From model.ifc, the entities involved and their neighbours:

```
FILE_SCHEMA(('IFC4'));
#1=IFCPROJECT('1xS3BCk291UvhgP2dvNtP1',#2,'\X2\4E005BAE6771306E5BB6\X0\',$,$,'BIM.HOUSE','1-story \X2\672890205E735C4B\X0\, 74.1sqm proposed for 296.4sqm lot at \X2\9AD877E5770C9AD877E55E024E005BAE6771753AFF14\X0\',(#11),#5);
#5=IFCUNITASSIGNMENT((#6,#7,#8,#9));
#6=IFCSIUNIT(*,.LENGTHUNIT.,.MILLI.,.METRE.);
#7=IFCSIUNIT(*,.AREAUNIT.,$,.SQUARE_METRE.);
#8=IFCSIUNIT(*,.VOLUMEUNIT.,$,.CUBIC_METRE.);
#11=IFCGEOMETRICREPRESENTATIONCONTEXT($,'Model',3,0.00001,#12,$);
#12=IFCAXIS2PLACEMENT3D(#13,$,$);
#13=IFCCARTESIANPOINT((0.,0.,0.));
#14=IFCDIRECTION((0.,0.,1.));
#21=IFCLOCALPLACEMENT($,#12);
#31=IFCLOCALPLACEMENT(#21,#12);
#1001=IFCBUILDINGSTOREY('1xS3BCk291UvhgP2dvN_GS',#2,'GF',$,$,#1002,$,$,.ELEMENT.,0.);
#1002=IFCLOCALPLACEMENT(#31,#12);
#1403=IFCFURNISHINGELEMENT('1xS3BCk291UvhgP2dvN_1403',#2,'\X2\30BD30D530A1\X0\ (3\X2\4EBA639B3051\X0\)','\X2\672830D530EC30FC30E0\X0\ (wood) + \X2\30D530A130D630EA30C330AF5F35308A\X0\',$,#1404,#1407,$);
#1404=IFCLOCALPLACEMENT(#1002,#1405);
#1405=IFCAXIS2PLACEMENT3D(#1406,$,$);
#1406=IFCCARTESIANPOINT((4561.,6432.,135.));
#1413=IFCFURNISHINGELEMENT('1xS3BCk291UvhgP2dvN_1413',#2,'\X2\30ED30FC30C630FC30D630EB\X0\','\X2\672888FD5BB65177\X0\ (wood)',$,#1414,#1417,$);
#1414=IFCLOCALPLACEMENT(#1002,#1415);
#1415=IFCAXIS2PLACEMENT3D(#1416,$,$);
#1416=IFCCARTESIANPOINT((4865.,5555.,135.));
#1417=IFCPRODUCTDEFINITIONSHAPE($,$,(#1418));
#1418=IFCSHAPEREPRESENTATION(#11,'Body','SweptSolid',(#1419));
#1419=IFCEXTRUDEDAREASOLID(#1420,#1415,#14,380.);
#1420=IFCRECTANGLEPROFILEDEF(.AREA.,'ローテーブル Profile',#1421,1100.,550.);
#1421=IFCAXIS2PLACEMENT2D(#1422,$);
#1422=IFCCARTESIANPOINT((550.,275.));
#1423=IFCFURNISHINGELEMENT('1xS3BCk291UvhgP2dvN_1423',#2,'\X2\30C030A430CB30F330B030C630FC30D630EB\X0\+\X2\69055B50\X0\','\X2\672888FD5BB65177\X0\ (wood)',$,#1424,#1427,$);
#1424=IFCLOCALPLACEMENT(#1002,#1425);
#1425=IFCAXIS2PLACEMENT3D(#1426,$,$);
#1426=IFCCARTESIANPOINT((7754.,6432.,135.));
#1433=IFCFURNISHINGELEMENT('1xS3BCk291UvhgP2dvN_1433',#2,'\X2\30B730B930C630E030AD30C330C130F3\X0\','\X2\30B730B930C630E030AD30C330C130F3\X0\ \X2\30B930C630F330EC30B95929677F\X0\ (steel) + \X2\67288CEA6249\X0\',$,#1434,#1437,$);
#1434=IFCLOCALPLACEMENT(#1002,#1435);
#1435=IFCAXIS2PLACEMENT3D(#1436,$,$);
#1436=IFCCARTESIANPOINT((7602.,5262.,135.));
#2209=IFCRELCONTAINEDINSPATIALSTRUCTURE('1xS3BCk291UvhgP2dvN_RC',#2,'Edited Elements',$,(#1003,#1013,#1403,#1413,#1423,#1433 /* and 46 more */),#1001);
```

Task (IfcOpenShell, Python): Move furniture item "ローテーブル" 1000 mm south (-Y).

```python
import ifcopenshell
import ifcopenshell.api.geometry
import ifcopenshell.util.placement

model = ifcopenshell.open("model.ifc")

item = model.by_guid("1xS3BCk291UvhgP2dvN_1413")
matrix = ifcopenshell.util.placement.get_local_placement(item.ObjectPlacement)
matrix[1, 3] -= 1000.0
ifcopenshell.api.geometry.edit_object_placement(model, product=item, matrix=matrix, is_si=False)

print(ifcopenshell.util.placement.get_local_placement(item.ObjectPlacement).round(3) + 0.0)

model.write("model_rev.ifc")
```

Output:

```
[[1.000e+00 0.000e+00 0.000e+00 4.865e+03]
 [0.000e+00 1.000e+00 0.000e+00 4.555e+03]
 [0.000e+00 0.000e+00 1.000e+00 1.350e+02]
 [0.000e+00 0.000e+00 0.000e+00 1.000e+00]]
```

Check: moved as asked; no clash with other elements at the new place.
